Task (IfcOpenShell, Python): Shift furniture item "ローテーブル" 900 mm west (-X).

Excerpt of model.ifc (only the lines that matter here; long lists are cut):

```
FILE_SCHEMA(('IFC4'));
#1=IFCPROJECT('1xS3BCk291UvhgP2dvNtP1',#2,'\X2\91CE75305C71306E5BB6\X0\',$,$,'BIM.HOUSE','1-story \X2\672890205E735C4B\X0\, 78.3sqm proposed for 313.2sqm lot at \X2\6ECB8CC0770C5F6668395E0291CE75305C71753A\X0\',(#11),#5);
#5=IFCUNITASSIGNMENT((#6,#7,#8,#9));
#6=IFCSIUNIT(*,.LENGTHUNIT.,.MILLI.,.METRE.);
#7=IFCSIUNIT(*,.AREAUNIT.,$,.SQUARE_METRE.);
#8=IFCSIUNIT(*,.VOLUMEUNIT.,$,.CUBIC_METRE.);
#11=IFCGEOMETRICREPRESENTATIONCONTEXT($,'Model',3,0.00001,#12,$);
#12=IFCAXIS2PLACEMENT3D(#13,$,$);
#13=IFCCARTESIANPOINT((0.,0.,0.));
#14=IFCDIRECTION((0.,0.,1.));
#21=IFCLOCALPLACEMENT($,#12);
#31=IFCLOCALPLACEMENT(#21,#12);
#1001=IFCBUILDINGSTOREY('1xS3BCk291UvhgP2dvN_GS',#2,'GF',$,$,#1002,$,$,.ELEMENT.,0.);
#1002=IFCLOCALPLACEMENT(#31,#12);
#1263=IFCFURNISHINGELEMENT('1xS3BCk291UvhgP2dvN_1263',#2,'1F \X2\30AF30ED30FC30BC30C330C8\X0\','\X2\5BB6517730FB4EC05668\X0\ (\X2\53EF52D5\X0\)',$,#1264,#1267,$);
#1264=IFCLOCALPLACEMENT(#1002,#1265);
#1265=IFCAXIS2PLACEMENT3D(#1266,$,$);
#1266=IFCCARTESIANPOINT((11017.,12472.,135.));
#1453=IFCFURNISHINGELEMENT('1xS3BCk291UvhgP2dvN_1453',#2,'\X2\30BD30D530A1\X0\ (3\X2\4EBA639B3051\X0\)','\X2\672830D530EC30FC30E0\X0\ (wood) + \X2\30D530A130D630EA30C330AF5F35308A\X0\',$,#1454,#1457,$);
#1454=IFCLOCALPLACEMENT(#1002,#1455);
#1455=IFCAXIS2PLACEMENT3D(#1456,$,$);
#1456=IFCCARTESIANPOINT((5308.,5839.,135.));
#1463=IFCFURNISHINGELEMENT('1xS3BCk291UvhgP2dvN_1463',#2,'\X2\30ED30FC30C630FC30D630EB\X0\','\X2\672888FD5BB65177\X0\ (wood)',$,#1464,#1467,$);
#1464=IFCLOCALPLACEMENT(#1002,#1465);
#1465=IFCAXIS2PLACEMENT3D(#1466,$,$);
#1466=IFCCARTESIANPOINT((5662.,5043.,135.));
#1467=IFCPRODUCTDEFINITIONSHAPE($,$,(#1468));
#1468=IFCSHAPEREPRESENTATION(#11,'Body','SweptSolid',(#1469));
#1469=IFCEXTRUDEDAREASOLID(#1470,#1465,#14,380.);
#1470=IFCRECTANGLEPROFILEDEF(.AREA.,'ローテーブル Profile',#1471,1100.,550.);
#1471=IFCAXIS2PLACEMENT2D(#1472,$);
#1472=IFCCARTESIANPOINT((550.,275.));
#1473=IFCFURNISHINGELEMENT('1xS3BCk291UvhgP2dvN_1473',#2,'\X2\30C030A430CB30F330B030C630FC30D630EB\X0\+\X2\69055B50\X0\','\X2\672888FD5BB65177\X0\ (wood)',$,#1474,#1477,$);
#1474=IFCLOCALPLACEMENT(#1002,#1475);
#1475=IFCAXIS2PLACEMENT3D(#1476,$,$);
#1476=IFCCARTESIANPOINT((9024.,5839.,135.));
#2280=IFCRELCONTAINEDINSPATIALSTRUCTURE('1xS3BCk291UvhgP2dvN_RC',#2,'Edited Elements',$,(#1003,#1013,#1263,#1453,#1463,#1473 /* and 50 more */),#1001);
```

```python
import ifcopenshell
import ifcopenshell.api.geometry
import ifcopenshell.util.placement

model = ifcopenshell.open("model.ifc")

item = model.by_id(1463)
matrix = ifcopenshell.util.placement.get_local_placement(item.ObjectPlacement)
matrix[0, 3] -= 900.0
ifcopenshell.api.geometry.edit_object_placement(model, product=item, matrix=matrix, is_si=False)

print(ifcopenshell.util.placement.get_local_placement(item.ObjectPlacement).round(3) + 0.0)

model.write("model_v2.ifc")
```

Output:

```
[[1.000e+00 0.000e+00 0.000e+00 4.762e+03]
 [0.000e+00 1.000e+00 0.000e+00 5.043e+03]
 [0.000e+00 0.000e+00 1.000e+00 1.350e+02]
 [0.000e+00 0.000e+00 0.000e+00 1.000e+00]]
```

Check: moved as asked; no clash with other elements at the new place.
